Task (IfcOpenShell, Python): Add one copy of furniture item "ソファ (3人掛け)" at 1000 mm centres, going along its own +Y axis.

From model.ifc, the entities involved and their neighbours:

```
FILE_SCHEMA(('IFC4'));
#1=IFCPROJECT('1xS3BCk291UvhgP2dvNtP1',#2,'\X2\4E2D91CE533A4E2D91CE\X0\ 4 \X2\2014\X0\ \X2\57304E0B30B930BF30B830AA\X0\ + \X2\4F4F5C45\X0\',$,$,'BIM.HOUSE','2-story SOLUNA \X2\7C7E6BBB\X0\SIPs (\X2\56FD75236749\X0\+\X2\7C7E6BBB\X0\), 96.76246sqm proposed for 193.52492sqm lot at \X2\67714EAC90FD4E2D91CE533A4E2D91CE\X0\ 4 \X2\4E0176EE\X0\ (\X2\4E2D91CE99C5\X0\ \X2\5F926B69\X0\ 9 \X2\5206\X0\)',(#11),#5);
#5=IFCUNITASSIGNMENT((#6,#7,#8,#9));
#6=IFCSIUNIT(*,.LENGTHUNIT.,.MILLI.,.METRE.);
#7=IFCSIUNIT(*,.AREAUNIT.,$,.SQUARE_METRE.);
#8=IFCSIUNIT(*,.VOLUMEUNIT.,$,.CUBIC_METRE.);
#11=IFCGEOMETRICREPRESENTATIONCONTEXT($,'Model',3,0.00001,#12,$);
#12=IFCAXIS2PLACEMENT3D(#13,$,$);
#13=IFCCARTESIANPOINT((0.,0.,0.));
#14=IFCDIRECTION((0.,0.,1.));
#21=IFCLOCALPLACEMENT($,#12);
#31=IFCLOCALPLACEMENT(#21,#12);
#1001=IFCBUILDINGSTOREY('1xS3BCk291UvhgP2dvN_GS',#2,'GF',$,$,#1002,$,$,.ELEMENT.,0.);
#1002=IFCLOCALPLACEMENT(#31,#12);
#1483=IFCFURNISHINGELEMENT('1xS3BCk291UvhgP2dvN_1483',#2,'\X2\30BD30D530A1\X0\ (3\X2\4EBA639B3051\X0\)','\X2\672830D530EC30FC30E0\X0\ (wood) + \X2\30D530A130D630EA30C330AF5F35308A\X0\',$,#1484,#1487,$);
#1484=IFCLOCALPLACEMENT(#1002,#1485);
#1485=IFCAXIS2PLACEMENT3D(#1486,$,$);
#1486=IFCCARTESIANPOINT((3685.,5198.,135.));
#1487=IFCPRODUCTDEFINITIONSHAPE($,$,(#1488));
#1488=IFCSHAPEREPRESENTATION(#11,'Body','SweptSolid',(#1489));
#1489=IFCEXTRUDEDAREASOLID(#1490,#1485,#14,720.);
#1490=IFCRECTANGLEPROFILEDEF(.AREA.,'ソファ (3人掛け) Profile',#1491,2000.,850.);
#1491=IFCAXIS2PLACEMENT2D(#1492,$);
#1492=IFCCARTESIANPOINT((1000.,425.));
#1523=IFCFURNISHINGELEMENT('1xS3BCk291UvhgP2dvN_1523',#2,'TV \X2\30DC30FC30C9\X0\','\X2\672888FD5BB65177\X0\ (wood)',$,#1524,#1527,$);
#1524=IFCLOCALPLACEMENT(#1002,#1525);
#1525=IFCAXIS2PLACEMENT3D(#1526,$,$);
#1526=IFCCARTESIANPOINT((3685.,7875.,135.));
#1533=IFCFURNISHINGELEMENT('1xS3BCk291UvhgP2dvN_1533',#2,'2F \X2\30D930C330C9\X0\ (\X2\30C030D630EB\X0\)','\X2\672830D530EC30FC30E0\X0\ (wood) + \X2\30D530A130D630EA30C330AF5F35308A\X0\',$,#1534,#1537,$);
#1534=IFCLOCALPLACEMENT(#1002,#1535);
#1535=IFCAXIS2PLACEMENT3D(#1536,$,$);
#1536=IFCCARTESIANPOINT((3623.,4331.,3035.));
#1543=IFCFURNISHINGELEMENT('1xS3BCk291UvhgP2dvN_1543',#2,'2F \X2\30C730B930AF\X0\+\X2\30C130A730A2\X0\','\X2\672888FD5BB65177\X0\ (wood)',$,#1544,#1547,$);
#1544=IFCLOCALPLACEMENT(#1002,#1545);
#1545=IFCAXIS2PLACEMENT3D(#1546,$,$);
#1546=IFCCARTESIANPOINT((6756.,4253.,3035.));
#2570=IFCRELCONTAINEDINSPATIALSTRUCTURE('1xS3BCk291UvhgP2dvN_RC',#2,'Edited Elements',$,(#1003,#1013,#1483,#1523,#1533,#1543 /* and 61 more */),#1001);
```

```python
import ifcopenshell
import ifcopenshell.api.geometry
import ifcopenshell.api.root
import ifcopenshell.util.element
import ifcopenshell.util.placement
import ifcopenshell.util.unit

model = ifcopenshell.open("model.ifc")
unit_scale = ifcopenshell.util.unit.calculate_unit_scale(model)


def reuse_history(source, copy):
    """copy_class also copies each property set's owner history, people and application; keep the originals."""
    for rel in copy.IsDefinedBy:
        if rel.is_a("IfcRelDefinesByProperties") and (history := rel.RelatingPropertyDefinition.OwnerHistory):
            rel.RelatingPropertyDefinition.OwnerHistory = source.OwnerHistory
            ifcopenshell.util.element.remove_deep2(model, history)


source = model.by_id(1483)
base = ifcopenshell.util.placement.get_local_placement(source.ObjectPlacement)
step = base[:3, 1] * 1 / unit_scale

for i in range(1, 2):
    copy = ifcopenshell.api.root.copy_class(model, product=source)
    copy.Representation = ifcopenshell.util.element.copy_deep(
        model, source.Representation, exclude=["IfcGeometricRepresentationContext", "IfcRepresentationMap"]
    )
    reuse_history(source, copy)
    matrix = base.copy()
    matrix[:3, 3] += i * step
    print("added at", matrix[:3, 3].round(3) + 0.0)
    ifcopenshell.api.geometry.edit_object_placement(model, product=copy, matrix=matrix, is_si=False)

model.write("model_rev.ifc")
```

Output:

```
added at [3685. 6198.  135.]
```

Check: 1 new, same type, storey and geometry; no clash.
